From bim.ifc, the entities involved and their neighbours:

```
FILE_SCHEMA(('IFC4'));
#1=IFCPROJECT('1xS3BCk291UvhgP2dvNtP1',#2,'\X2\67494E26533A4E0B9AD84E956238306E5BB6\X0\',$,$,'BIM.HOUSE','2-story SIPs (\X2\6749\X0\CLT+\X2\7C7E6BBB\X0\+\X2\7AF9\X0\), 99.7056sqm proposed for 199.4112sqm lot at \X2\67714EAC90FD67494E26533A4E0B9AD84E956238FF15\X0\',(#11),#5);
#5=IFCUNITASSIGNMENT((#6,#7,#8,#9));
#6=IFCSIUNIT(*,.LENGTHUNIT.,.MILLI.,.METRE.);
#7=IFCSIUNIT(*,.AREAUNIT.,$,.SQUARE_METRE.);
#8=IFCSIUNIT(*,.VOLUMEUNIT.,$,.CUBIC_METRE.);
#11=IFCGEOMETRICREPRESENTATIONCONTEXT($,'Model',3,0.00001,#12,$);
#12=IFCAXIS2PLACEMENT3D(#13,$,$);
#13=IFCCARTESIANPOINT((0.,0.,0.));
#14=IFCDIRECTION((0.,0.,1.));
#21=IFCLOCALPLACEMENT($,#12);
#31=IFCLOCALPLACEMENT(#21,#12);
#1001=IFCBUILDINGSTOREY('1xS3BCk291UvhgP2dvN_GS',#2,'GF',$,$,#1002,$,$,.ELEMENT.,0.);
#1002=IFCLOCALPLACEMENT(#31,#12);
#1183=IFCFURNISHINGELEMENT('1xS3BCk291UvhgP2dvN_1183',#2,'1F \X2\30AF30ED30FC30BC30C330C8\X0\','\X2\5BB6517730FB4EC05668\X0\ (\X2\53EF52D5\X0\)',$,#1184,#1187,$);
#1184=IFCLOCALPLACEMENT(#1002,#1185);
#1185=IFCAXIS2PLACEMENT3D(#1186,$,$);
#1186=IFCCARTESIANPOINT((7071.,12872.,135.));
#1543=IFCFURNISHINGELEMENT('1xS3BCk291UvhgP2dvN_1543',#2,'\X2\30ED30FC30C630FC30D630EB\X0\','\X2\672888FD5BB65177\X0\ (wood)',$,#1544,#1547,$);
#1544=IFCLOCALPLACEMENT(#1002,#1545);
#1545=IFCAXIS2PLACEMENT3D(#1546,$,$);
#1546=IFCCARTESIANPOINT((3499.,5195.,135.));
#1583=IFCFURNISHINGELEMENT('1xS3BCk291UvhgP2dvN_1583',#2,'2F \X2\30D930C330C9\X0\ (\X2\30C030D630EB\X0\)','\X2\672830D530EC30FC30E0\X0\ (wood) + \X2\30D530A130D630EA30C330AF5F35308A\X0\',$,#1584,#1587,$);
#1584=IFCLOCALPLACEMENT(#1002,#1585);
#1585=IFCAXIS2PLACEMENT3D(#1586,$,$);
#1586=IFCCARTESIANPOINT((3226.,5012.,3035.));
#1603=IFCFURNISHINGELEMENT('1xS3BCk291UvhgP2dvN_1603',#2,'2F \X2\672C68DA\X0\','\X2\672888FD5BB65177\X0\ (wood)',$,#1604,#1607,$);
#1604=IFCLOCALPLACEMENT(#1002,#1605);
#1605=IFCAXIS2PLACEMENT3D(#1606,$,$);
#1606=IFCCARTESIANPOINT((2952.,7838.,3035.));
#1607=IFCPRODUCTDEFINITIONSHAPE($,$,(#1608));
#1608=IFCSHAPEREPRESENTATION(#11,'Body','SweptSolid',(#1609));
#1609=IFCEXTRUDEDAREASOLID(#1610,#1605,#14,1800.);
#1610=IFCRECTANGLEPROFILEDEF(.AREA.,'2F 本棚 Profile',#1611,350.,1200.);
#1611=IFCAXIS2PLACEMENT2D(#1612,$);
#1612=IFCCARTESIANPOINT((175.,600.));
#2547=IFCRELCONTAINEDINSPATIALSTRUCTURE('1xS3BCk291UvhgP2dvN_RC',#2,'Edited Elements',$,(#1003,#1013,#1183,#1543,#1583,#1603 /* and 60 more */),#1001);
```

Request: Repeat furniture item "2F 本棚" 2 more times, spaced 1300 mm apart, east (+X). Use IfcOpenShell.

```python
import numpy as np
import ifcopenshell
import ifcopenshell.api.geometry
import ifcopenshell.api.root
import ifcopenshell.util.element
import ifcopenshell.util.placement

model = ifcopenshell.open("bim.ifc")


def reuse_history(source, copy):
    """copy_class also copies each property set's owner history, people and application; keep the originals."""
    for rel in copy.IsDefinedBy:
        if rel.is_a("IfcRelDefinesByProperties") and (history := rel.RelatingPropertyDefinition.OwnerHistory):
            rel.RelatingPropertyDefinition.OwnerHistory = source.OwnerHistory
            ifcopenshell.util.element.remove_deep2(model, history)


source = model.by_id(1603)
base = ifcopenshell.util.placement.get_local_placement(source.ObjectPlacement)
step = np.array([1.0, 0.0, 0.0]) * 1300.0

for i in range(1, 3):
    copy = ifcopenshell.api.root.copy_class(model, product=source)
    copy.Representation = ifcopenshell.util.element.copy_deep(
        model, source.Representation, exclude=["IfcGeometricRepresentationContext", "IfcRepresentationMap"]
    )
    reuse_history(source, copy)
    matrix = base.copy()
    matrix[:3, 3] += i * step
    print("added at", matrix[:3, 3].round(3) + 0.0)
    ifcopenshell.api.geometry.edit_object_placement(model, product=copy, matrix=matrix, is_si=False)

model.write("bim-out.ifc")
```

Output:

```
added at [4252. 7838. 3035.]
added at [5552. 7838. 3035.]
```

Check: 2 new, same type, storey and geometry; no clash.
